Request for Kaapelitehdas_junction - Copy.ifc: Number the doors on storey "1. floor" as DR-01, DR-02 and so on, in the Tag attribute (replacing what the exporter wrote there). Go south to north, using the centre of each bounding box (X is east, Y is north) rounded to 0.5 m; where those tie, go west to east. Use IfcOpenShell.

First a look at what the model holds.

```python
import ifcopenshell
import ifcopenshell.util.element
import ifcopenshell.util.placement

model = ifcopenshell.open("Kaapelitehdas_junction - Copy.ifc")
print(model.schema)
storey = next(s for s in model.by_type("IfcBuildingStorey") if s.Name == "1. floor")
doors = [e for e in ifcopenshell.util.element.get_decomposition(storey) if e.is_a("IfcDoor")]
for e in sorted(doors, key=lambda e: e.id()):
    origin = ifcopenshell.util.placement.get_local_placement(e.ObjectPlacement)[:3, 3]
    print(e.id(), e.Tag, e.Name, origin.round(2) + 0.0, sep=" | ")
```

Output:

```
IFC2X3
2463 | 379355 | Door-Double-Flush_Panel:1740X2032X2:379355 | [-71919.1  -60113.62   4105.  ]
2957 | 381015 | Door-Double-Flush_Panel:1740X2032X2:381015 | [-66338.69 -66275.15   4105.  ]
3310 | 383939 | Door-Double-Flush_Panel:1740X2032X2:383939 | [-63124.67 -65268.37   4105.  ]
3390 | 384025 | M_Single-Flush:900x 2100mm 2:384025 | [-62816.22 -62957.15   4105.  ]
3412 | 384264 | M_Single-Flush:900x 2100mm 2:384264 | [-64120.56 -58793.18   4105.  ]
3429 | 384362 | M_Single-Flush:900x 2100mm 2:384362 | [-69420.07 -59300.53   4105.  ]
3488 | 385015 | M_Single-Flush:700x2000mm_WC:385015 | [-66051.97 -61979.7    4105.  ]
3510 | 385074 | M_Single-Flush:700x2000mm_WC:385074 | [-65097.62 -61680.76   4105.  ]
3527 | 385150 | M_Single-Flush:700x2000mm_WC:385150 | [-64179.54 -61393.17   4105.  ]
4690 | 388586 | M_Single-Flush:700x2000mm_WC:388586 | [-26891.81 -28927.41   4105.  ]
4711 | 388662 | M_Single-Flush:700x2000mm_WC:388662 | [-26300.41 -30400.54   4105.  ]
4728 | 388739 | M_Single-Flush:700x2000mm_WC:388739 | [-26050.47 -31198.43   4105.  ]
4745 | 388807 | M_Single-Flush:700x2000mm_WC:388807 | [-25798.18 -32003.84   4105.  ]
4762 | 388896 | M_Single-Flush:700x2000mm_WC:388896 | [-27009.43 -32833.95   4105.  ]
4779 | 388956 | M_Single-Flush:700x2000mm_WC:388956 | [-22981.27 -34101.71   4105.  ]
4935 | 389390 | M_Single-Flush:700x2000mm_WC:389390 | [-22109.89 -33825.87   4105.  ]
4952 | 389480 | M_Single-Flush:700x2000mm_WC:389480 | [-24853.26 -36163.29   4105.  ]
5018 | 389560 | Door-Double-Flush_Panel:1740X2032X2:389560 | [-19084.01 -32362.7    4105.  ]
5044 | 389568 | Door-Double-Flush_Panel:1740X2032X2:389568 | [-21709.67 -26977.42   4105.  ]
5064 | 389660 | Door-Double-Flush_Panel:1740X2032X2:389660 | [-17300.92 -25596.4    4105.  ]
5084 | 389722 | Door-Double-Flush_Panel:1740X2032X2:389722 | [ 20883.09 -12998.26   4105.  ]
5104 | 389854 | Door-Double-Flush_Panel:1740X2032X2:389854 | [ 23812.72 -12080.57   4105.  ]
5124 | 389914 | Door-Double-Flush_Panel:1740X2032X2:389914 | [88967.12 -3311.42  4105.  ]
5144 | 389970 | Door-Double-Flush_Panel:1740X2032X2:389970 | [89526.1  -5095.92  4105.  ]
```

```python
import ifcopenshell
import ifcopenshell.geom
import ifcopenshell.util.element
import ifcopenshell.util.shape

model = ifcopenshell.open("Kaapelitehdas_junction - Copy.ifc")
settings = ifcopenshell.geom.settings()
settings.set("use-world-coords", True)


def centre(element):
    shape = ifcopenshell.geom.create_shape(settings, element)
    return ifcopenshell.util.shape.get_bbox_centroid(shape.geometry)


storey = next(s for s in model.by_type("IfcBuildingStorey") if s.Name == "1. floor")
doors = [e for e in ifcopenshell.util.element.get_decomposition(storey) if e.is_a("IfcDoor")]

# Insertion points can sit at a corner or the storey origin, so sort by the geometry (in metres).
centres = {e: centre(e) for e in doors}
doors.sort(key=lambda e: (round(centres[e][1] / 0.5), centres[e][0]))

for i, e in enumerate(doors, start=1):
    number = f"DR-{i:02d}"
    e.Tag = number
    print(e.id(), number)

model.write("Kaapelitehdas_junction - Copy_edited.ifc")
```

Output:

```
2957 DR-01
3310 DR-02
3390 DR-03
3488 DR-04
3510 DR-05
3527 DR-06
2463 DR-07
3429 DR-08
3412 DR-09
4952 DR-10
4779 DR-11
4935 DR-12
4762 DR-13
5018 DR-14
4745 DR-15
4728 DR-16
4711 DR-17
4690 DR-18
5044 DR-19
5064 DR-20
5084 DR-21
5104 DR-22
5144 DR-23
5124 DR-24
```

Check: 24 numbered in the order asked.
